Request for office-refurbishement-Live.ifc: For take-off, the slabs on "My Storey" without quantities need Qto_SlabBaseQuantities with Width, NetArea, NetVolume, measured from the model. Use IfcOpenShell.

First a look at what the model holds.

```python
import ifcopenshell
import ifcopenshell.util.element
import ifcopenshell.util.unit

model = ifcopenshell.open("office-refurbishement-Live.ifc")
print(model.schema)
for unit_type in ("LENGTHUNIT", "AREAUNIT", "VOLUMEUNIT"):
    print(unit_type, ifcopenshell.util.unit.calculate_unit_scale(model, unit_type))
storey = next(s for s in model.by_type("IfcBuildingStorey") if s.Name == "My Storey")
slabs = [e for e in ifcopenshell.util.element.get_decomposition(storey) if e.is_a("IfcSlab")]
for e in sorted(slabs, key=lambda e: e.id()):
    print(e.id(), e.is_a(), e.Name, list(ifcopenshell.util.element.get_psets(e, qtos_only=True)), sep=" | ")
```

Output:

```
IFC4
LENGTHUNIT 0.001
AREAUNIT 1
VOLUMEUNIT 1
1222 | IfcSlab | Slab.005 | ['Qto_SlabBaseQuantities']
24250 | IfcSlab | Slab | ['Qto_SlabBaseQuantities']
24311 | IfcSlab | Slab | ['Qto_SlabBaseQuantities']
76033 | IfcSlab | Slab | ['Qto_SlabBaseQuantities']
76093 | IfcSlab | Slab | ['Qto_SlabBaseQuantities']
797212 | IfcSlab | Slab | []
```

```python
import ifcopenshell
import ifcopenshell.api.pset
import ifcopenshell.geom
import ifcopenshell.util.element
import ifcopenshell.util.shape
import ifcopenshell.util.unit

model = ifcopenshell.open("office-refurbishement-Live.ifc")
unit_scale = ifcopenshell.util.unit.calculate_unit_scale(model)
area_scale = ifcopenshell.util.unit.calculate_unit_scale(model, "AREAUNIT")
volume_scale = ifcopenshell.util.unit.calculate_unit_scale(model, "VOLUMEUNIT")
settings = ifcopenshell.geom.settings()

storey = next(s for s in model.by_type("IfcBuildingStorey") if s.Name == "My Storey")
slabs = [e for e in ifcopenshell.util.element.get_decomposition(storey) if e.is_a("IfcSlab")]

for e in sorted(slabs, key=lambda e: e.id()):
    if ifcopenshell.util.element.get_psets(e, qtos_only=True, should_inherit=False):
        continue
    # Geometry comes back in metres, in the element's own axes.
    shape = ifcopenshell.geom.create_shape(settings, e)
    values = {
        "Width": ifcopenshell.util.shape.get_z(shape.geometry) / unit_scale,
        "NetArea": ifcopenshell.util.shape.get_footprint_area(shape.geometry) / area_scale,
        "NetVolume": ifcopenshell.util.shape.get_volume(shape.geometry) / volume_scale,
    }
    qto = ifcopenshell.api.pset.add_qto(model, product=e, name="Qto_SlabBaseQuantities")
    ifcopenshell.api.pset.edit_qto(model, qto=qto, properties=values)
    print(e.id(), {k: round(v, 3) for k, v in values.items()})

model.write("office-refurbishement-Live-out.ifc")
```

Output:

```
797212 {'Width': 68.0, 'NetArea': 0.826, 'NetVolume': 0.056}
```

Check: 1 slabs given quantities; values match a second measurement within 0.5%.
